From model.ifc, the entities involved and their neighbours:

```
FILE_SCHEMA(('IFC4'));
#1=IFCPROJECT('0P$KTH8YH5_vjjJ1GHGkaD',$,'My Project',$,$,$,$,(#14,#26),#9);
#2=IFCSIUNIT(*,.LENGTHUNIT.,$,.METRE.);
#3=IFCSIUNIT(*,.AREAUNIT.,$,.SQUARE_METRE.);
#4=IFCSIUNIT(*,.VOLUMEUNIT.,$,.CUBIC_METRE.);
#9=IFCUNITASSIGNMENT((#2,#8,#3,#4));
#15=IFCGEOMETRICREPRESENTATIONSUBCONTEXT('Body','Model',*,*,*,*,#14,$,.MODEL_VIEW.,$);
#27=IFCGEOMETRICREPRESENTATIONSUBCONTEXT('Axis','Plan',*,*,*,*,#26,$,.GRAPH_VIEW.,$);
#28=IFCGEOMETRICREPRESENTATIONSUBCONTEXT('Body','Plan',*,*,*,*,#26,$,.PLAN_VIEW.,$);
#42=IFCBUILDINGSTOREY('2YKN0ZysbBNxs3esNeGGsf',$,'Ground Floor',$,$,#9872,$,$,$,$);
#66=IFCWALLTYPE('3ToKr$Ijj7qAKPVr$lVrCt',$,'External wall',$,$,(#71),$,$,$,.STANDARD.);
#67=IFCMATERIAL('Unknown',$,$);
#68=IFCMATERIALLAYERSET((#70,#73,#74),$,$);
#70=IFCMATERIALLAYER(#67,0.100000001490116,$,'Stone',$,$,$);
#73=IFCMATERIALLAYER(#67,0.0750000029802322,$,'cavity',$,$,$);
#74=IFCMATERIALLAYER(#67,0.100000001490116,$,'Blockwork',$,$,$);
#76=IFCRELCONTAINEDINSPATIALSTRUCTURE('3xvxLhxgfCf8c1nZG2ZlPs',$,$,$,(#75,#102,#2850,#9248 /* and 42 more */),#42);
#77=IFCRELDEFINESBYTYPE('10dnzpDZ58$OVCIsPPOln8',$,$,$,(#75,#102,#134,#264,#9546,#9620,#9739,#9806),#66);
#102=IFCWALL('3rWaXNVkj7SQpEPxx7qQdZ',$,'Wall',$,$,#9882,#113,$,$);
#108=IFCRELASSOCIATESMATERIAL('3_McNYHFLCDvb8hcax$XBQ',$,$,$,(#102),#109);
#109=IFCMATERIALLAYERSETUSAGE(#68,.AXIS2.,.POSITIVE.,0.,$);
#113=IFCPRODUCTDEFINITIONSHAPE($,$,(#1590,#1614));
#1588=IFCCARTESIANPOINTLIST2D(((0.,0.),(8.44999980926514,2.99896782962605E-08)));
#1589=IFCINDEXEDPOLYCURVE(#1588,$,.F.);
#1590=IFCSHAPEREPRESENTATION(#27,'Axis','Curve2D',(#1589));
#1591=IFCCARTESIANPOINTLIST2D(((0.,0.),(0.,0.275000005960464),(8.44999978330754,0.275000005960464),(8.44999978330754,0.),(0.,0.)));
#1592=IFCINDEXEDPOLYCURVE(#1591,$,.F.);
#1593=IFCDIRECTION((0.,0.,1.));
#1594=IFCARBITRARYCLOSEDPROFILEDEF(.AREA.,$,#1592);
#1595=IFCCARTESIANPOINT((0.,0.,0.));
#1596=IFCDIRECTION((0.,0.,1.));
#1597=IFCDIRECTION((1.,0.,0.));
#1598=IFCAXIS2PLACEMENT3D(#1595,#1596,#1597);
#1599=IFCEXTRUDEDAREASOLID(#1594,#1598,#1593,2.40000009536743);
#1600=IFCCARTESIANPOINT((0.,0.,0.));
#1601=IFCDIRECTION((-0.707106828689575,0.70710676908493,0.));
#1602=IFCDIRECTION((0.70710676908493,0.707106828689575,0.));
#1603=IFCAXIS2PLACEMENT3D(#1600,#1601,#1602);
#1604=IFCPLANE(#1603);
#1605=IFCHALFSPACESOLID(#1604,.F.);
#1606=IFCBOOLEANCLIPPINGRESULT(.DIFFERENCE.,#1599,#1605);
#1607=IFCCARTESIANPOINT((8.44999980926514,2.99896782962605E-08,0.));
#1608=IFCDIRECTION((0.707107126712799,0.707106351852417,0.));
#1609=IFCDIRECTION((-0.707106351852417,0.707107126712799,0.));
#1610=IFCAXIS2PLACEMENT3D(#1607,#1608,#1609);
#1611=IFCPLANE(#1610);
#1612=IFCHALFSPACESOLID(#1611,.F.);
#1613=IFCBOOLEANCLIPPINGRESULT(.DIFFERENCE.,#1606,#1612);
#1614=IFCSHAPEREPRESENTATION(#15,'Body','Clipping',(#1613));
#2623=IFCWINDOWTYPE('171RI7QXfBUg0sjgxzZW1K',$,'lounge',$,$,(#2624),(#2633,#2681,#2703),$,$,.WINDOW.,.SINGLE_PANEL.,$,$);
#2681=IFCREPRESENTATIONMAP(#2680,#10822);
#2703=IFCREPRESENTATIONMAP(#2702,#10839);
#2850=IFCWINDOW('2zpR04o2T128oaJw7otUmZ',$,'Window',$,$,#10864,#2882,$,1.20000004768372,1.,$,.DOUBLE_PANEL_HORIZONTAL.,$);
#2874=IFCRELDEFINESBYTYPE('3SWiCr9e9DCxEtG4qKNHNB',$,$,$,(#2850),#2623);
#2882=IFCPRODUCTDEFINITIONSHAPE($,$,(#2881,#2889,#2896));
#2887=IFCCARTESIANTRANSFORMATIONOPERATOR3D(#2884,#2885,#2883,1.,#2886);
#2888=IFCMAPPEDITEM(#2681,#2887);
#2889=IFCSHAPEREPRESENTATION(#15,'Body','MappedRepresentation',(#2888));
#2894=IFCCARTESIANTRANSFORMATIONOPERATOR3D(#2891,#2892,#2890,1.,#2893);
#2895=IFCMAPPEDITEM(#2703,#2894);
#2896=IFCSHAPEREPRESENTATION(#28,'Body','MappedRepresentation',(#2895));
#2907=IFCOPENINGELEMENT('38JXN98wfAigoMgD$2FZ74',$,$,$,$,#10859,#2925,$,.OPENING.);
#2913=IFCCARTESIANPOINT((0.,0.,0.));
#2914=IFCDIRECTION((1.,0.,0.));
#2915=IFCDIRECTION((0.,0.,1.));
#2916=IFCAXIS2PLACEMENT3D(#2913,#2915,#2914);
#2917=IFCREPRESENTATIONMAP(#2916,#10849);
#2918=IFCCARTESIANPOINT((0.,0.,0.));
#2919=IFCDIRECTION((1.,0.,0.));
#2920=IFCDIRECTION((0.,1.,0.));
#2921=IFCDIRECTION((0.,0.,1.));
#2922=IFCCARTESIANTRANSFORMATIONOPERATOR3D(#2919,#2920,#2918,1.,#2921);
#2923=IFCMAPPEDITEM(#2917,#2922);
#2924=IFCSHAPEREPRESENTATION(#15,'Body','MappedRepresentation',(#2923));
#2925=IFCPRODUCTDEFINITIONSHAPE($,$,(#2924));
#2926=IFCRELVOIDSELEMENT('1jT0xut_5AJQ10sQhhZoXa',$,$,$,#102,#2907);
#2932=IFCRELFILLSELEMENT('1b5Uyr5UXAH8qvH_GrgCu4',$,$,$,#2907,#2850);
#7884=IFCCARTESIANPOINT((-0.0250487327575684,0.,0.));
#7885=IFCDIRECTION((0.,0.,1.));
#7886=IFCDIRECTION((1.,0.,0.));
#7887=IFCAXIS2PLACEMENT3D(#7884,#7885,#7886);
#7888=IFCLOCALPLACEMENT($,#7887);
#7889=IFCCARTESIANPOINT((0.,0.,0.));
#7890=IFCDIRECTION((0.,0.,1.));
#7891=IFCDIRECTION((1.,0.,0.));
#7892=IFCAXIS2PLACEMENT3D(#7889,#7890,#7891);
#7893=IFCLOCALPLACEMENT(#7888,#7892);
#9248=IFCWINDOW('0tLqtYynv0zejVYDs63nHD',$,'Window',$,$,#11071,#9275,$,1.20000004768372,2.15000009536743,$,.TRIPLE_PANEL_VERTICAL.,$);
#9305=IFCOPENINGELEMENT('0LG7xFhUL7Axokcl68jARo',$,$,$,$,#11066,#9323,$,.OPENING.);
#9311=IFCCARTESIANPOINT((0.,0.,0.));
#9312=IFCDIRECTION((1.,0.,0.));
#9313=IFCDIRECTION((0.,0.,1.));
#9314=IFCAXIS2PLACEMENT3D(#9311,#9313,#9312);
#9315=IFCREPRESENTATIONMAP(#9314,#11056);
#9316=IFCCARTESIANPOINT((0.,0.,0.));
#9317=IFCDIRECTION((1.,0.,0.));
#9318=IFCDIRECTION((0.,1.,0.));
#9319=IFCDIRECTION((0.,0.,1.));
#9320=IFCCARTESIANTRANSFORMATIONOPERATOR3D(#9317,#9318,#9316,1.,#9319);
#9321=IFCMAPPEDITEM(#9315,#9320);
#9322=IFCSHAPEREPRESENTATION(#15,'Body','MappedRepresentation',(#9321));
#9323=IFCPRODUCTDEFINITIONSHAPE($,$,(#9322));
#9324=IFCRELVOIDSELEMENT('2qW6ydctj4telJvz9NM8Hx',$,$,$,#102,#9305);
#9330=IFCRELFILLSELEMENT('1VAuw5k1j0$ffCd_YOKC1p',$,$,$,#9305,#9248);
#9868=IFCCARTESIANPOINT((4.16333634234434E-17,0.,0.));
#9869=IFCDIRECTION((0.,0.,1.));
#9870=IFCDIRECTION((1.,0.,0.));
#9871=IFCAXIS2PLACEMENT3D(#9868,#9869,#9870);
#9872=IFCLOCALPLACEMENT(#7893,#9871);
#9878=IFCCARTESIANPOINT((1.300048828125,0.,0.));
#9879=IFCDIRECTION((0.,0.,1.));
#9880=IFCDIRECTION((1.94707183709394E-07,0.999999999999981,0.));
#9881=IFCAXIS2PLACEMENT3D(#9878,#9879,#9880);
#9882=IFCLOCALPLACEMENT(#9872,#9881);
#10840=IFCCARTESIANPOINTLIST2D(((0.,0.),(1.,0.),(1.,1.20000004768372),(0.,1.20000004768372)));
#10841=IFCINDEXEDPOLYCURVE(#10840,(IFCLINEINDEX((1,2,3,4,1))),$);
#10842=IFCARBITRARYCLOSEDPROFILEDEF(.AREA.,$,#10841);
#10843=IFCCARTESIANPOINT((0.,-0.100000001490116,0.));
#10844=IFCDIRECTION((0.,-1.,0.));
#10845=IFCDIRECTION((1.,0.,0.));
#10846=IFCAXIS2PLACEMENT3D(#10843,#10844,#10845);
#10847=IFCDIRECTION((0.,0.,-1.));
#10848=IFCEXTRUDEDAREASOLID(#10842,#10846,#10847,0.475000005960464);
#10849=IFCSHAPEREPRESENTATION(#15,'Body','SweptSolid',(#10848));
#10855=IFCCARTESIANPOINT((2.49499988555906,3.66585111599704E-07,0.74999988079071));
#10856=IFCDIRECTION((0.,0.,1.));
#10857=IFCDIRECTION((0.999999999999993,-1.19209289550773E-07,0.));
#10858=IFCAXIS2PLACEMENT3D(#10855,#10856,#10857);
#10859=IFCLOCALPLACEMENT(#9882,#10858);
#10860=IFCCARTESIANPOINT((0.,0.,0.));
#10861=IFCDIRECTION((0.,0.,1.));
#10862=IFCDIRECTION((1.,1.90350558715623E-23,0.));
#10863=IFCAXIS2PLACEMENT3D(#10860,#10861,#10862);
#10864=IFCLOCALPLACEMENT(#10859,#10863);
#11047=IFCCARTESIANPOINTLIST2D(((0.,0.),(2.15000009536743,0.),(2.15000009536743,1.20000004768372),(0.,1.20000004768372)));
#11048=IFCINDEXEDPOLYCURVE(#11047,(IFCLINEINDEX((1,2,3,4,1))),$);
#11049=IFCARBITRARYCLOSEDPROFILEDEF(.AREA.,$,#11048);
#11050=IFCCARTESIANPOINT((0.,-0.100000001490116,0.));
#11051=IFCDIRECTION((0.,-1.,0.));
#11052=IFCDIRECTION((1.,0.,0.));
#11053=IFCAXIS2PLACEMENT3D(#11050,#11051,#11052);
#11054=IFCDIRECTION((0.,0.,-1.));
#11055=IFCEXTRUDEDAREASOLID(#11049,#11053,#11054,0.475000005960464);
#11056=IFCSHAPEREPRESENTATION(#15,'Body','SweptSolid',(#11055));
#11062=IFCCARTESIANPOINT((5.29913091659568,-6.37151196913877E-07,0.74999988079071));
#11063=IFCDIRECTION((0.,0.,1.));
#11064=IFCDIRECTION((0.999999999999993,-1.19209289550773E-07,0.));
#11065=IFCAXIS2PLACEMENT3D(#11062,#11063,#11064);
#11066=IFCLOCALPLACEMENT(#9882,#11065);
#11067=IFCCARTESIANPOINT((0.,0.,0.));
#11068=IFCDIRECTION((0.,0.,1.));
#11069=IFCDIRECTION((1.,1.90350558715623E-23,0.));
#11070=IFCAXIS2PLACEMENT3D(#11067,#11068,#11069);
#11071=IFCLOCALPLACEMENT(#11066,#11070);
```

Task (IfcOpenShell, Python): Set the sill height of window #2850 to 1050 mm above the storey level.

```python
import numpy as np
import ifcopenshell
import ifcopenshell.api.geometry
import ifcopenshell.geom
import ifcopenshell.util.element
import ifcopenshell.util.placement
import ifcopenshell.util.shape
import ifcopenshell.util.unit

model = ifcopenshell.open("model.ifc")
unit_scale = ifcopenshell.util.unit.calculate_unit_scale(model)

window = model.by_guid("2zpR04o2T128oaJw7otUmZ")
opening = window.FillsVoids[0].RelatingOpeningElement
storey = ifcopenshell.util.element.get_container(window, ifc_class="IfcBuildingStorey")
level = ifcopenshell.util.placement.get_local_placement(storey.ObjectPlacement)[2, 3]

# The opening's origin need not be at the sill, so measure its lowest point.
shape = ifcopenshell.geom.create_shape(ifcopenshell.geom.settings(), opening)
bottom = ifcopenshell.util.shape.get_shape_bottom_elevation(shape, shape.geometry) / unit_scale
dz = level + 1.05 / unit_scale - bottom

shift = np.array([0.0, 0.0, dz])
# The window is placed relative to its opening, so it follows when the opening moves.
matrix = ifcopenshell.util.placement.get_local_placement(opening.ObjectPlacement)
matrix[:3, 3] += shift
ifcopenshell.api.geometry.edit_object_placement(
    model, product=opening, matrix=matrix, is_si=False, should_transform_children=True
)

print(f"moved by {dz * unit_scale:+.3f} m")

model.write("model_rev.ifc")
```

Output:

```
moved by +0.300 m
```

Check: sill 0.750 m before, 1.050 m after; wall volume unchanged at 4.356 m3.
